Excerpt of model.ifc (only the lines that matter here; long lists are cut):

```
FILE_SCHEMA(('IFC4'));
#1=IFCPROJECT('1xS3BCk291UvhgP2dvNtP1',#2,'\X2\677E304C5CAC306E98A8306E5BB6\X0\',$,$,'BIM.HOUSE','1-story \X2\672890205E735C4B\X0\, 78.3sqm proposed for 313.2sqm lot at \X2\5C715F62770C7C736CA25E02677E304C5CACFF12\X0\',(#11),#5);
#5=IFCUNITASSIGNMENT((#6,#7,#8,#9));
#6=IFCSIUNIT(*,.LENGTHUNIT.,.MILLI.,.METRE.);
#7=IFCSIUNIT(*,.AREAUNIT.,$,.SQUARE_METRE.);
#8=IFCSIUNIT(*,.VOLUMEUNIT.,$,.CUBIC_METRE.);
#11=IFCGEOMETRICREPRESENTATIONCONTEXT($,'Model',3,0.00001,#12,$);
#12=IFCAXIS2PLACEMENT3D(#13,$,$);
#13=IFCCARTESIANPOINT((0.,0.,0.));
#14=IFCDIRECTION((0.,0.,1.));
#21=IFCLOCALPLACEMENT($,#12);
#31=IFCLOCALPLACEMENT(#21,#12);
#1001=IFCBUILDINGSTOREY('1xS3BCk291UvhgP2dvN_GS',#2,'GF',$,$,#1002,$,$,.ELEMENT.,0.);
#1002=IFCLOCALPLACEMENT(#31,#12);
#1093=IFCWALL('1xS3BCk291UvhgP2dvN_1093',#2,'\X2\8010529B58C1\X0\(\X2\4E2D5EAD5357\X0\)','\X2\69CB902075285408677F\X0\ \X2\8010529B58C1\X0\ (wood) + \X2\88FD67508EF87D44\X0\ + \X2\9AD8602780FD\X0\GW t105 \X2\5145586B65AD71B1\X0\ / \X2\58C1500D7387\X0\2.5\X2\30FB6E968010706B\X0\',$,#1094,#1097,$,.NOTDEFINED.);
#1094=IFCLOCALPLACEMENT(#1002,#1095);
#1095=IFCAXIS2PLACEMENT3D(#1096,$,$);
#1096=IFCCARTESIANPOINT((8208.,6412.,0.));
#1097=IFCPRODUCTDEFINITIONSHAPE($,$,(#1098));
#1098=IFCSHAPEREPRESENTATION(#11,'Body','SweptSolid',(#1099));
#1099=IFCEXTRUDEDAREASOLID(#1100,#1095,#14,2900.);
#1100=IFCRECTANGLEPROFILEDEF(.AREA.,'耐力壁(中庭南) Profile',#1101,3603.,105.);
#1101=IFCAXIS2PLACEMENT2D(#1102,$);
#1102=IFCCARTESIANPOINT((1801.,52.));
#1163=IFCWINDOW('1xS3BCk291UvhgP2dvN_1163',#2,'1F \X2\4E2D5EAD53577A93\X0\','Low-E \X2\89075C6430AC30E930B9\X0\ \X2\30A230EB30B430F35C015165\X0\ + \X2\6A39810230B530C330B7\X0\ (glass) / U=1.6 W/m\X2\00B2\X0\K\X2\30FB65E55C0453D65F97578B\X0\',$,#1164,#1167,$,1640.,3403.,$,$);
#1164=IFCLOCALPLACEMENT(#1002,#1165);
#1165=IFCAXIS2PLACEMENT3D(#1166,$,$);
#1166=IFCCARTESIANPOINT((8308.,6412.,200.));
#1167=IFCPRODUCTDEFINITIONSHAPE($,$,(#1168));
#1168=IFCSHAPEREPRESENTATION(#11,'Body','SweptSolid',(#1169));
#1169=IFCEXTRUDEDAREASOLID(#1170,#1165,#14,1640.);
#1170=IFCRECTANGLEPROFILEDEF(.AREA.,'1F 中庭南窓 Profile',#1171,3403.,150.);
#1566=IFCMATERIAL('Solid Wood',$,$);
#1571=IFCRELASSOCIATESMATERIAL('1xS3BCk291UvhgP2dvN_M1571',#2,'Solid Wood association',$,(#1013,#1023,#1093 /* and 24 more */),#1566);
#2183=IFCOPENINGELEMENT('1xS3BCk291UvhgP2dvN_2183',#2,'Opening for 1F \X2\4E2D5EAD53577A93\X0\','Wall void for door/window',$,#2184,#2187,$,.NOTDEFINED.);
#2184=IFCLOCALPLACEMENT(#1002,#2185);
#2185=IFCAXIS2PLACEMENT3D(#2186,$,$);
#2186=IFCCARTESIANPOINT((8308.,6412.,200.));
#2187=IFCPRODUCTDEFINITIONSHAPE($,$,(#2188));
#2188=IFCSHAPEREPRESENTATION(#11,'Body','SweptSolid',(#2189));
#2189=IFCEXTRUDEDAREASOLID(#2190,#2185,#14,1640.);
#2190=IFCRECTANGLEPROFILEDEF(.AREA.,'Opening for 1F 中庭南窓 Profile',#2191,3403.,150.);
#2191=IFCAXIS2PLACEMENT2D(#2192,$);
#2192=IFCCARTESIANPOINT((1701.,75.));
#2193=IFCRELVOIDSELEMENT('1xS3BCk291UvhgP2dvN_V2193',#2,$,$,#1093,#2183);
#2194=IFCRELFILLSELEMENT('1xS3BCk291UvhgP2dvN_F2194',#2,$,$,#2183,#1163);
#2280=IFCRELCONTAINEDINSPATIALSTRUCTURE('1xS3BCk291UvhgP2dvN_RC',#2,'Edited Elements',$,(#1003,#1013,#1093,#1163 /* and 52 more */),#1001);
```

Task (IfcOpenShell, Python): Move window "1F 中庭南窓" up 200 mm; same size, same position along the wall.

```python
import numpy as np
import ifcopenshell
import ifcopenshell.api.geometry
import ifcopenshell.util.placement
import ifcopenshell.util.unit

model = ifcopenshell.open("model.ifc")
unit_scale = ifcopenshell.util.unit.calculate_unit_scale(model)

window = model.by_guid("1xS3BCk291UvhgP2dvN_1163")
opening = window.FillsVoids[0].RelatingOpeningElement
dz = 200.0

shift = np.array([0.0, 0.0, dz])
# The window is not placed relative to its opening, so move both.
for product in (opening, window):
    matrix = ifcopenshell.util.placement.get_local_placement(product.ObjectPlacement)
    matrix[:3, 3] += shift
    ifcopenshell.api.geometry.edit_object_placement(model, product=product, matrix=matrix, is_si=False)

print(f"moved by {dz * unit_scale:+.3f} m")

model.write("model_edited.ifc")
```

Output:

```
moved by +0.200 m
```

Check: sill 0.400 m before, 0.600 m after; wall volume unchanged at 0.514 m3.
